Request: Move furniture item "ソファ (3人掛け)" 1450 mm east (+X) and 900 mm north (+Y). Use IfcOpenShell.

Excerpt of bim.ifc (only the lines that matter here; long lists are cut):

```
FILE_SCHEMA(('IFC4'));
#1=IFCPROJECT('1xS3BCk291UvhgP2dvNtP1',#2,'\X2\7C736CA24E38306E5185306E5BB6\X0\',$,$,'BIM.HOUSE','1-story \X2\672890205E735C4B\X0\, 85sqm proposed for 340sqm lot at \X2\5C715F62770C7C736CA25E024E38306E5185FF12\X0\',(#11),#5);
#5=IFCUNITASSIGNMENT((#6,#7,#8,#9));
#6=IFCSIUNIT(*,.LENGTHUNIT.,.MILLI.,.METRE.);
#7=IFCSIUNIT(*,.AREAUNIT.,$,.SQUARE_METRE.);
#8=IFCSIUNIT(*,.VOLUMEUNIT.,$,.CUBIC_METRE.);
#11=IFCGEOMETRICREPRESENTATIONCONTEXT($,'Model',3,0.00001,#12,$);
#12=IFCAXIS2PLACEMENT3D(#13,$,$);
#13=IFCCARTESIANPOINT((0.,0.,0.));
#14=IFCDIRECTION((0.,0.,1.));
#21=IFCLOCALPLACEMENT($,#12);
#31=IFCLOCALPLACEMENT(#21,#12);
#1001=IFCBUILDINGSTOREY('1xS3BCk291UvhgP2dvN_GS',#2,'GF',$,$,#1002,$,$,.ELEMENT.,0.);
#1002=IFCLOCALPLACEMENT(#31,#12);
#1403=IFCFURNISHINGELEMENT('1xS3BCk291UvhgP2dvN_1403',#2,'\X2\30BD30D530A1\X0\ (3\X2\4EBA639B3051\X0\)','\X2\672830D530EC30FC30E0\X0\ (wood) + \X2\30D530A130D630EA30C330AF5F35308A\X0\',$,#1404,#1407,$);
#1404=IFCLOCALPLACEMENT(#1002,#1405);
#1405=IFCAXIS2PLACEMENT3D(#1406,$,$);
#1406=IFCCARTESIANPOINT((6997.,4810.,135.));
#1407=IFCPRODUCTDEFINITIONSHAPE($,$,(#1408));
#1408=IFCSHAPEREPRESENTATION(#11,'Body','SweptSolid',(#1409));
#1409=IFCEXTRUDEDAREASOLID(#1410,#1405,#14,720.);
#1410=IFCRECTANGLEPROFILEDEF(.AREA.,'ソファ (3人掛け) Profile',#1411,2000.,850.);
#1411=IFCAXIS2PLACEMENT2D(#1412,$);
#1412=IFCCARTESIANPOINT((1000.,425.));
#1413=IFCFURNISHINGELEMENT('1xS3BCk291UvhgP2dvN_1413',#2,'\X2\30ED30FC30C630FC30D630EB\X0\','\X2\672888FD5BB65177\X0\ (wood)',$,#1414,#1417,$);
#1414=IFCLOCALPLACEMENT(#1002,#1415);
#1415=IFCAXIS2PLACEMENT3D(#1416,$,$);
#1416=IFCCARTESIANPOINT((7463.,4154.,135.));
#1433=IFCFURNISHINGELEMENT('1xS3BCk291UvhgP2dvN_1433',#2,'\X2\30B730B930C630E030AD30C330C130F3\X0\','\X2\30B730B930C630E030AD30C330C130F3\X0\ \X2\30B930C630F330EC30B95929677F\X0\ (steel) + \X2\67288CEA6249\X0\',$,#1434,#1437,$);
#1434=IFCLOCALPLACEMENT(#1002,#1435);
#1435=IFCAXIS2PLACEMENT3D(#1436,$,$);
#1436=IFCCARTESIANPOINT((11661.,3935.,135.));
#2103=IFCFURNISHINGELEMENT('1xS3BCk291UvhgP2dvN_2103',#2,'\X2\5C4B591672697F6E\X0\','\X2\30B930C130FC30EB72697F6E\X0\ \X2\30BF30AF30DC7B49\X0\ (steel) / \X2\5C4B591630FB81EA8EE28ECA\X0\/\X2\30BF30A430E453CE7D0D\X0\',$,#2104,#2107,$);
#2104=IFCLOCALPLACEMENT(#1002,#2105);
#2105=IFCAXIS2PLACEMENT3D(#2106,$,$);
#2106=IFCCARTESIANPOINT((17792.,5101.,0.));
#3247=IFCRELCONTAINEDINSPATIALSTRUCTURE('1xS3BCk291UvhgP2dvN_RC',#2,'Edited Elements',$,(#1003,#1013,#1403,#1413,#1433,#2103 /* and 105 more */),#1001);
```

```python
import ifcopenshell
import ifcopenshell.api.geometry
import ifcopenshell.util.placement
import ifcopenshell.util.unit

model = ifcopenshell.open("bim.ifc")
unit_scale = ifcopenshell.util.unit.calculate_unit_scale(model)

item = model.by_id(1403)
matrix = ifcopenshell.util.placement.get_local_placement(item.ObjectPlacement)
matrix[0, 3] += 1.45 / unit_scale
matrix[1, 3] += 0.9 / unit_scale
ifcopenshell.api.geometry.edit_object_placement(model, product=item, matrix=matrix, is_si=False)

print(ifcopenshell.util.placement.get_local_placement(item.ObjectPlacement).round(3) + 0.0)

model.write("bim-out.ifc")
```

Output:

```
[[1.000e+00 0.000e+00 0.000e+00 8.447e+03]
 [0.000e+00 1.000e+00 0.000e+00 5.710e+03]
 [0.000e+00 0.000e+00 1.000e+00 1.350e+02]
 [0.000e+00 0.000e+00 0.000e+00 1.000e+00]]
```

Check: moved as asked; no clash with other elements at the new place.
